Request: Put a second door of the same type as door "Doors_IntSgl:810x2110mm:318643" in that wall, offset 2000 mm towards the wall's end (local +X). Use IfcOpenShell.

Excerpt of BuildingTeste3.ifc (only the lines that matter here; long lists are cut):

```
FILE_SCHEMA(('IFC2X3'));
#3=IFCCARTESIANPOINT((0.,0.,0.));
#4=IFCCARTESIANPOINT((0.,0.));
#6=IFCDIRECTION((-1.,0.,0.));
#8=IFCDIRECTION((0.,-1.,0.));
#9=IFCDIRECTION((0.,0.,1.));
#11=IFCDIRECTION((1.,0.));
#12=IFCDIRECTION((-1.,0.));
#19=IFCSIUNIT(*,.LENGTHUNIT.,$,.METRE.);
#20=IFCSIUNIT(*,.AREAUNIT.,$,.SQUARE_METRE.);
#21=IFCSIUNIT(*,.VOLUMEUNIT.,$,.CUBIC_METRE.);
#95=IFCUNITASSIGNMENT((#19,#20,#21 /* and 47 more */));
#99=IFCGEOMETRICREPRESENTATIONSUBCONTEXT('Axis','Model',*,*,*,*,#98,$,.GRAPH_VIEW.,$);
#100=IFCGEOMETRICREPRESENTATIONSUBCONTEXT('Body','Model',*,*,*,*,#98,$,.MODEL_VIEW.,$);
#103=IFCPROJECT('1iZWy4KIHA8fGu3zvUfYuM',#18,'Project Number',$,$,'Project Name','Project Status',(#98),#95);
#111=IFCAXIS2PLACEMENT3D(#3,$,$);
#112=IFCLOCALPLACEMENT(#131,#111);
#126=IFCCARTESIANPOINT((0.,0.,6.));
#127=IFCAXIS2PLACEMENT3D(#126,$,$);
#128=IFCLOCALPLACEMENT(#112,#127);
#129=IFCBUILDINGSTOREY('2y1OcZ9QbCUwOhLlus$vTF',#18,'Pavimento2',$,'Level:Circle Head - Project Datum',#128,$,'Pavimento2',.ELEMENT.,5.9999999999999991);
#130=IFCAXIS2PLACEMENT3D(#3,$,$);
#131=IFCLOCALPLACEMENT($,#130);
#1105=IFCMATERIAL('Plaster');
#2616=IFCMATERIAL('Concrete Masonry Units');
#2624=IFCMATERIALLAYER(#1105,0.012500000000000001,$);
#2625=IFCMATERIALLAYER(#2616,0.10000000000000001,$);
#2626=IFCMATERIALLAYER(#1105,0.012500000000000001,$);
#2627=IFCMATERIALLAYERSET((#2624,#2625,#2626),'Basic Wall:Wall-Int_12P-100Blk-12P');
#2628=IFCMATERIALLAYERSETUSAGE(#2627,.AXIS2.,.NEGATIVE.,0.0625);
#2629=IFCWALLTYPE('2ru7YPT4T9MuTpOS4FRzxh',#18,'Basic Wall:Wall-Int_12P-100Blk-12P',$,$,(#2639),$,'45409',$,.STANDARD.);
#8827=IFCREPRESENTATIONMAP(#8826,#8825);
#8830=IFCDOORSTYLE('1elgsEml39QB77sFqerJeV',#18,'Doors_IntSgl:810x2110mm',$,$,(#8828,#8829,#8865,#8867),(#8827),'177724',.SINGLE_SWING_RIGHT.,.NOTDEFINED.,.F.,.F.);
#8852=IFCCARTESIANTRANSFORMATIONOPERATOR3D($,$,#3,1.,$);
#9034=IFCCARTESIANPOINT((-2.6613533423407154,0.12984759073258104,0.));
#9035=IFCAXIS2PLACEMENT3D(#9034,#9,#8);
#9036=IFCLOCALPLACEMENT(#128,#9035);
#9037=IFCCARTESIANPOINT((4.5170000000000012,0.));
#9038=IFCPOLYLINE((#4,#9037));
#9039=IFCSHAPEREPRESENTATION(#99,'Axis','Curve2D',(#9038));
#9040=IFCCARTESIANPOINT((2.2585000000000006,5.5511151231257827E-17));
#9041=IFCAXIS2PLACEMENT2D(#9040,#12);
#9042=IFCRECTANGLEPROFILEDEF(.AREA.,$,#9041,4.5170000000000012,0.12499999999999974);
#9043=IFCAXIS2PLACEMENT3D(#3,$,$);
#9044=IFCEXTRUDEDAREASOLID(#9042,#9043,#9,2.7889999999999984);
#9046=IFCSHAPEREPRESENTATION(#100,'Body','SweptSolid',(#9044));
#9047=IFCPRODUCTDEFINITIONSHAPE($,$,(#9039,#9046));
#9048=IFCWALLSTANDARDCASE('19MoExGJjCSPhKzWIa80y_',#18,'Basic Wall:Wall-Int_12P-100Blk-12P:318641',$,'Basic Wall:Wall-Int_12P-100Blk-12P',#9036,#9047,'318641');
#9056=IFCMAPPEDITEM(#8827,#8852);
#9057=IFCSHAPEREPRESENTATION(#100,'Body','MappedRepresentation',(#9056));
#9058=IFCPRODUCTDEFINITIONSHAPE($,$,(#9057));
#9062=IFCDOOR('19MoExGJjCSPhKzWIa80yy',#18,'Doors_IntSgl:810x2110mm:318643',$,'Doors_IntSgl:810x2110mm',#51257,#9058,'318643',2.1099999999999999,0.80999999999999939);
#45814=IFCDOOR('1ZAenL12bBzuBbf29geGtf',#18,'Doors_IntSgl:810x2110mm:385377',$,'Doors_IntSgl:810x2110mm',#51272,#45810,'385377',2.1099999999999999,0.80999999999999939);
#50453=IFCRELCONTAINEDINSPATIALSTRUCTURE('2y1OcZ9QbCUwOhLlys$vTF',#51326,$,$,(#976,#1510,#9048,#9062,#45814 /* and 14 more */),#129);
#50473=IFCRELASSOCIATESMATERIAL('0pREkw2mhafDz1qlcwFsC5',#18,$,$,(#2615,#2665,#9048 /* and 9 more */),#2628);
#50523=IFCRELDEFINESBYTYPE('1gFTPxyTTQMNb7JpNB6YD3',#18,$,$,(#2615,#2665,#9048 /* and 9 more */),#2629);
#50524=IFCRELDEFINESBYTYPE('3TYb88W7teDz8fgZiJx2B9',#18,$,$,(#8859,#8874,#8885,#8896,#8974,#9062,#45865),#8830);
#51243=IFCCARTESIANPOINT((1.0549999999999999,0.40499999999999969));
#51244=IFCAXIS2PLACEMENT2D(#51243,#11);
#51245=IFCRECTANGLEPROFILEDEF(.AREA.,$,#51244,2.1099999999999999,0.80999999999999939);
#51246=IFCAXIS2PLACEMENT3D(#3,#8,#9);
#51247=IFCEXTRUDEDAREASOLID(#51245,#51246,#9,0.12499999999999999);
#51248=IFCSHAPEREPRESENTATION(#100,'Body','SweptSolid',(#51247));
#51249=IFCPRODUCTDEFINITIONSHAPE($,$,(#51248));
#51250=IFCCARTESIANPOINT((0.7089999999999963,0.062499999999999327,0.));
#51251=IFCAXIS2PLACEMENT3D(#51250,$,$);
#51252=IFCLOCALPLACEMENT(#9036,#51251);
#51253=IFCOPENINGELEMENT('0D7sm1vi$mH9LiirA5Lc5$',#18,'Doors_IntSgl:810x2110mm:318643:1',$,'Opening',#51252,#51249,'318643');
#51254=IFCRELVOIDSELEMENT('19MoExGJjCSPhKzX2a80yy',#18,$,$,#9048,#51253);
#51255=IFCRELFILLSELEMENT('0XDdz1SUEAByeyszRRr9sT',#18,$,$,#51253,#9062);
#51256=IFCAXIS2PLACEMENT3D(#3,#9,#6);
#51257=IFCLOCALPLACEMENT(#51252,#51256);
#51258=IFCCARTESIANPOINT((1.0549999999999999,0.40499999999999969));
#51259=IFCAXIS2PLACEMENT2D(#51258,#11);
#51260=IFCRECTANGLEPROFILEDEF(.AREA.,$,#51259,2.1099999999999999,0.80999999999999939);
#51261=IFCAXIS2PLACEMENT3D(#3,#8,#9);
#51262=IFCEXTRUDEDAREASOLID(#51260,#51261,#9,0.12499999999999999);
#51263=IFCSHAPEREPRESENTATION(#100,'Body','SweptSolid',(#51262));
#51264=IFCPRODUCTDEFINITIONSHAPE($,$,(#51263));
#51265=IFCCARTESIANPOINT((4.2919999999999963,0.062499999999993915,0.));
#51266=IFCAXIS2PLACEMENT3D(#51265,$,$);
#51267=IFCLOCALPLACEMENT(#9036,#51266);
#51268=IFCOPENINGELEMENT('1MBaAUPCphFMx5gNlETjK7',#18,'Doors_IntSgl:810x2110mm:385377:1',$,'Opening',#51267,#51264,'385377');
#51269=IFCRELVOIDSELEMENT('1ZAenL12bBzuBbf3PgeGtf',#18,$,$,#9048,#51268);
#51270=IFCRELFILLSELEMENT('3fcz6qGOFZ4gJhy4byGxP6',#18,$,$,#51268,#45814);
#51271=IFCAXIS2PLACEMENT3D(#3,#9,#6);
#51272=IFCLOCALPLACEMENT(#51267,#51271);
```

```python
import ifcopenshell
import ifcopenshell.api.feature
import ifcopenshell.api.geometry
import ifcopenshell.api.root
import ifcopenshell.geom
import ifcopenshell.util.element
import ifcopenshell.util.placement
import ifcopenshell.util.shape

model = ifcopenshell.open("BuildingTeste3.ifc")
settings = ifcopenshell.geom.settings()


def volume(element):
    """Net volume in cubic metres, openings subtracted."""
    shape = ifcopenshell.geom.create_shape(settings, element)
    return ifcopenshell.util.shape.get_volume(shape.geometry)


def reuse_history(source, copy):
    """copy_class also copies each property set's owner history, people and application; keep the originals."""
    for rel in copy.IsDefinedBy:
        if rel.is_a("IfcRelDefinesByProperties") and (history := rel.RelatingPropertyDefinition.OwnerHistory):
            rel.RelatingPropertyDefinition.OwnerHistory = source.OwnerHistory
            ifcopenshell.util.element.remove_deep2(model, history)


door = model.by_id(9062)
opening = door.FillsVoids[0].RelatingOpeningElement
wall = opening.VoidsElements[0].RelatingBuildingElement
before = volume(wall)
shift = ifcopenshell.util.placement.get_local_placement(wall.ObjectPlacement)[:3, 0] * 2.0

# copy_class copies the void relationship, type, container and properties, but no geometry.
new_opening = ifcopenshell.api.root.copy_class(model, product=opening)
new_opening.Representation = ifcopenshell.util.element.copy_deep(
    model, opening.Representation, exclude=["IfcGeometricRepresentationContext", "IfcRepresentationMap"]
)
new_opening.Name = "Doors_IntSgl:810x2110mm"
new_opening.Tag = None
new_door = ifcopenshell.api.root.copy_class(model, product=door)
new_door.Representation = ifcopenshell.util.element.copy_deep(
    model, door.Representation, exclude=["IfcGeometricRepresentationContext", "IfcRepresentationMap"]
)
new_door.Name = "Doors_IntSgl:810x2110mm"
new_door.Tag = None
reuse_history(door, new_door)
fills = ifcopenshell.api.feature.add_filling(model, opening=new_opening, element=new_door)
fills.OwnerHistory = new_door.OwnerHistory  # required in IFC2X3

for old, new in ((opening, new_opening), (door, new_door)):
    matrix = ifcopenshell.util.placement.get_local_placement(old.ObjectPlacement)
    matrix[:3, 3] += shift
    ifcopenshell.api.geometry.edit_object_placement(model, product=new, matrix=matrix, is_si=False)

after = volume(wall)

print(f"wall volume {before:.3f} -> {after:.3f} m3")

model.write("BuildingTeste3_updated.ifc")
```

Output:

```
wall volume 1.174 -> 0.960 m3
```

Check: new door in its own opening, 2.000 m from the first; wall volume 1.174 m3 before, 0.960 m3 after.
